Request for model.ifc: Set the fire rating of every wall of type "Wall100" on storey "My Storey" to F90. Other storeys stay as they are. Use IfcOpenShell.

First a look at what the model holds.

```python
import ifcopenshell
import ifcopenshell.util.element

model = ifcopenshell.open("model.ifc")
print(model.schema)
storey = next(s for s in model.by_type("IfcBuildingStorey") if s.Name == "My Storey")
walls = [e for e in ifcopenshell.util.element.get_decomposition(storey) if e.is_a("IfcWall")]
seen = {}
for e in walls:
    element_type = ifcopenshell.util.element.get_type(e)
    key = (element_type.Name if element_type != e and element_type else None, ifcopenshell.util.element.get_pset(e, "Pset_WallCommon", "FireRating"))
    seen[key] = seen.get(key, 0) + 1
for (name, value), count in sorted(seen.items(), key=str):
    print(count, "x", name, "|", value)
```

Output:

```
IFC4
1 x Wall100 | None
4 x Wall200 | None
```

```python
import ifcopenshell
import ifcopenshell.api.pset
import ifcopenshell.util.element

model = ifcopenshell.open("model.ifc")

storey = next(s for s in model.by_type("IfcBuildingStorey") if s.Name == "My Storey")
walls = [e for e in ifcopenshell.util.element.get_decomposition(storey) if e.is_a("IfcWall")]

count = 0
for e in walls:
    element_type = ifcopenshell.util.element.get_type(e)
    if element_type in (None, e) or element_type.Name != "Wall100":
        continue
    # add_pset returns the element's existing set when there is one.
    pset = ifcopenshell.api.pset.add_pset(model, product=e, name="Pset_WallCommon")
    ifcopenshell.api.pset.edit_pset(model, pset=pset, properties={"FireRating": "F90"})
    count += 1

print(count, "walls updated")

model.write("model-out.ifc")
```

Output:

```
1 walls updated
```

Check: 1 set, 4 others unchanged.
